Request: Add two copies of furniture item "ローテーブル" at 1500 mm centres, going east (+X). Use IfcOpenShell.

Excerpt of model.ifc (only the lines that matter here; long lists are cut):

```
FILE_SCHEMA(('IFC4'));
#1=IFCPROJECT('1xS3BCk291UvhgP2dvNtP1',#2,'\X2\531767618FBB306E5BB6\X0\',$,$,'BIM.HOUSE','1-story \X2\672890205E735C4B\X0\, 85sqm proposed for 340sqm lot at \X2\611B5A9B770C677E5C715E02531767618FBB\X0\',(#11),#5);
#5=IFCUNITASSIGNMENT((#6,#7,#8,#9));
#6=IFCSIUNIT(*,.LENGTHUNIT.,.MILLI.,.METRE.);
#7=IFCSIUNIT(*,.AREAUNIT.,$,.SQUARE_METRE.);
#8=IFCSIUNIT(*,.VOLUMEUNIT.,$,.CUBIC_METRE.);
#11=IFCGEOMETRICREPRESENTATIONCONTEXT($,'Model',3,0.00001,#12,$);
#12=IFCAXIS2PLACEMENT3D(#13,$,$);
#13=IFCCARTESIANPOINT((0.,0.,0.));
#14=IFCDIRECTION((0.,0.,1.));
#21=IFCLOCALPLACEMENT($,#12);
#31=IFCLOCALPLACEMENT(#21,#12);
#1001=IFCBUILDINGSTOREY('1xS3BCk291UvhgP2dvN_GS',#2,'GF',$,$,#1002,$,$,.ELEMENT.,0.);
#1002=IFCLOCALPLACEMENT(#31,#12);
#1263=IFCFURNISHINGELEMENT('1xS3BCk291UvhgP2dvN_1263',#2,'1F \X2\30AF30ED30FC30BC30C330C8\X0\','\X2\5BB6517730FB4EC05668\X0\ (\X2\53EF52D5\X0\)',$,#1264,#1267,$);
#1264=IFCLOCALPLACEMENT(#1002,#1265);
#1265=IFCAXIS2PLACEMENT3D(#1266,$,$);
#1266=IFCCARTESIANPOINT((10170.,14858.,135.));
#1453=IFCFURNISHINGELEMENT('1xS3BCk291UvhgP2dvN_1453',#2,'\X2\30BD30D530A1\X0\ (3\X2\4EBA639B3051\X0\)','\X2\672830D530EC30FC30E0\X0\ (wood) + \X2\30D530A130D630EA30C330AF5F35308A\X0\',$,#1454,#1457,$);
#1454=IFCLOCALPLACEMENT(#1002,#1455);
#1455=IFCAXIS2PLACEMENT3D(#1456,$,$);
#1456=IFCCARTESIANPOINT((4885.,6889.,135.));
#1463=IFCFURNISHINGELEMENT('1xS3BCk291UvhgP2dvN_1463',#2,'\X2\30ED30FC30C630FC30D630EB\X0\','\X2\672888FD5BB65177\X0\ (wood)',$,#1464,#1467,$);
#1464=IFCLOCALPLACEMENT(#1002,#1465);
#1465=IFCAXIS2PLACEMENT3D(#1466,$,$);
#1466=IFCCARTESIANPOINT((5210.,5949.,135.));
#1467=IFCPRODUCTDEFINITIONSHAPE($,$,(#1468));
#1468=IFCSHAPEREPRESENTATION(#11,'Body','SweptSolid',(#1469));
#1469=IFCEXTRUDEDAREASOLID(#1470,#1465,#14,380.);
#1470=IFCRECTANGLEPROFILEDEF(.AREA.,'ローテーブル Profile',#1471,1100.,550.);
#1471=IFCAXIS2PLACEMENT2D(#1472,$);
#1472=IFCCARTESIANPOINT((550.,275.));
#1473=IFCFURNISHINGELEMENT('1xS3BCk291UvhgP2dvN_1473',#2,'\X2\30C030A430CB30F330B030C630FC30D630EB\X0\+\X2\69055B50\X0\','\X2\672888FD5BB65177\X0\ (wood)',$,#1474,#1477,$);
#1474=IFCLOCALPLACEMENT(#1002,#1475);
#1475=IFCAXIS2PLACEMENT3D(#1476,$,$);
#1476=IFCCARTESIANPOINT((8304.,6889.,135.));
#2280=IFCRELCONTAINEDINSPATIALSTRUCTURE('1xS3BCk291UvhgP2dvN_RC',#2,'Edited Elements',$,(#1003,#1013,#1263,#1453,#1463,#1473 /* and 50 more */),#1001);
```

```python
import numpy as np
import ifcopenshell
import ifcopenshell.api.geometry
import ifcopenshell.api.root
import ifcopenshell.util.element
import ifcopenshell.util.placement

model = ifcopenshell.open("model.ifc")


def reuse_history(source, copy):
    """copy_class also copies each property set's owner history, people and application; keep the originals."""
    for rel in copy.IsDefinedBy:
        if rel.is_a("IfcRelDefinesByProperties") and (history := rel.RelatingPropertyDefinition.OwnerHistory):
            rel.RelatingPropertyDefinition.OwnerHistory = source.OwnerHistory
            ifcopenshell.util.element.remove_deep2(model, history)


source = model.by_guid("1xS3BCk291UvhgP2dvN_1463")
base = ifcopenshell.util.placement.get_local_placement(source.ObjectPlacement)
step = np.array([1.0, 0.0, 0.0]) * 1500.0

for i in range(1, 3):
    copy = ifcopenshell.api.root.copy_class(model, product=source)
    copy.Representation = ifcopenshell.util.element.copy_deep(
        model, source.Representation, exclude=["IfcGeometricRepresentationContext", "IfcRepresentationMap"]
    )
    reuse_history(source, copy)
    matrix = base.copy()
    matrix[:3, 3] += i * step
    print("added at", matrix[:3, 3].round(3) + 0.0)
    ifcopenshell.api.geometry.edit_object_placement(model, product=copy, matrix=matrix, is_si=False)

model.write("model_edited.ifc")
```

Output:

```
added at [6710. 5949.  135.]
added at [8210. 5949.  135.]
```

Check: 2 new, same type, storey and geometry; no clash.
